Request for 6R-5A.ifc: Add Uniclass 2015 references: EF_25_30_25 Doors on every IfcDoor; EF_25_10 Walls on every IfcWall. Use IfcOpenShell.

First a look at what the model holds.

```python
import ifcopenshell

model = ifcopenshell.open("6R-5A.ifc")
print(model.schema)
print("classifications:", [c.Name for c in model.by_type("IfcClassification")])
for ifc_class in ("IfcDoor", "IfcRoof", "IfcStair", "IfcWall", "IfcWindow"):
    print(ifc_class, len(model.by_type(ifc_class)))
```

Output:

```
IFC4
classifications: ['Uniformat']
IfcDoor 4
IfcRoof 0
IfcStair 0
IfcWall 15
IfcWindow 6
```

```python
import ifcopenshell
import ifcopenshell.api.classification

model = ifcopenshell.open("6R-5A.ifc")

system = ifcopenshell.api.classification.add_classification(model, classification="Uniclass 2015")

codes = {
    "IfcDoor": ("EF_25_30_25", "Doors"),
    "IfcWall": ("EF_25_10", "Walls"),
}
for ifc_class, (code, name) in codes.items():
    products = model.by_type(ifc_class)
    ifcopenshell.api.classification.add_reference(
        model, products=products, classification=system, identification=code, name=name
    )
    print(code, len(products))

model.write("6R-5A_edited.ifc")
```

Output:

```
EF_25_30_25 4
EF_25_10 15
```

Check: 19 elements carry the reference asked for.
